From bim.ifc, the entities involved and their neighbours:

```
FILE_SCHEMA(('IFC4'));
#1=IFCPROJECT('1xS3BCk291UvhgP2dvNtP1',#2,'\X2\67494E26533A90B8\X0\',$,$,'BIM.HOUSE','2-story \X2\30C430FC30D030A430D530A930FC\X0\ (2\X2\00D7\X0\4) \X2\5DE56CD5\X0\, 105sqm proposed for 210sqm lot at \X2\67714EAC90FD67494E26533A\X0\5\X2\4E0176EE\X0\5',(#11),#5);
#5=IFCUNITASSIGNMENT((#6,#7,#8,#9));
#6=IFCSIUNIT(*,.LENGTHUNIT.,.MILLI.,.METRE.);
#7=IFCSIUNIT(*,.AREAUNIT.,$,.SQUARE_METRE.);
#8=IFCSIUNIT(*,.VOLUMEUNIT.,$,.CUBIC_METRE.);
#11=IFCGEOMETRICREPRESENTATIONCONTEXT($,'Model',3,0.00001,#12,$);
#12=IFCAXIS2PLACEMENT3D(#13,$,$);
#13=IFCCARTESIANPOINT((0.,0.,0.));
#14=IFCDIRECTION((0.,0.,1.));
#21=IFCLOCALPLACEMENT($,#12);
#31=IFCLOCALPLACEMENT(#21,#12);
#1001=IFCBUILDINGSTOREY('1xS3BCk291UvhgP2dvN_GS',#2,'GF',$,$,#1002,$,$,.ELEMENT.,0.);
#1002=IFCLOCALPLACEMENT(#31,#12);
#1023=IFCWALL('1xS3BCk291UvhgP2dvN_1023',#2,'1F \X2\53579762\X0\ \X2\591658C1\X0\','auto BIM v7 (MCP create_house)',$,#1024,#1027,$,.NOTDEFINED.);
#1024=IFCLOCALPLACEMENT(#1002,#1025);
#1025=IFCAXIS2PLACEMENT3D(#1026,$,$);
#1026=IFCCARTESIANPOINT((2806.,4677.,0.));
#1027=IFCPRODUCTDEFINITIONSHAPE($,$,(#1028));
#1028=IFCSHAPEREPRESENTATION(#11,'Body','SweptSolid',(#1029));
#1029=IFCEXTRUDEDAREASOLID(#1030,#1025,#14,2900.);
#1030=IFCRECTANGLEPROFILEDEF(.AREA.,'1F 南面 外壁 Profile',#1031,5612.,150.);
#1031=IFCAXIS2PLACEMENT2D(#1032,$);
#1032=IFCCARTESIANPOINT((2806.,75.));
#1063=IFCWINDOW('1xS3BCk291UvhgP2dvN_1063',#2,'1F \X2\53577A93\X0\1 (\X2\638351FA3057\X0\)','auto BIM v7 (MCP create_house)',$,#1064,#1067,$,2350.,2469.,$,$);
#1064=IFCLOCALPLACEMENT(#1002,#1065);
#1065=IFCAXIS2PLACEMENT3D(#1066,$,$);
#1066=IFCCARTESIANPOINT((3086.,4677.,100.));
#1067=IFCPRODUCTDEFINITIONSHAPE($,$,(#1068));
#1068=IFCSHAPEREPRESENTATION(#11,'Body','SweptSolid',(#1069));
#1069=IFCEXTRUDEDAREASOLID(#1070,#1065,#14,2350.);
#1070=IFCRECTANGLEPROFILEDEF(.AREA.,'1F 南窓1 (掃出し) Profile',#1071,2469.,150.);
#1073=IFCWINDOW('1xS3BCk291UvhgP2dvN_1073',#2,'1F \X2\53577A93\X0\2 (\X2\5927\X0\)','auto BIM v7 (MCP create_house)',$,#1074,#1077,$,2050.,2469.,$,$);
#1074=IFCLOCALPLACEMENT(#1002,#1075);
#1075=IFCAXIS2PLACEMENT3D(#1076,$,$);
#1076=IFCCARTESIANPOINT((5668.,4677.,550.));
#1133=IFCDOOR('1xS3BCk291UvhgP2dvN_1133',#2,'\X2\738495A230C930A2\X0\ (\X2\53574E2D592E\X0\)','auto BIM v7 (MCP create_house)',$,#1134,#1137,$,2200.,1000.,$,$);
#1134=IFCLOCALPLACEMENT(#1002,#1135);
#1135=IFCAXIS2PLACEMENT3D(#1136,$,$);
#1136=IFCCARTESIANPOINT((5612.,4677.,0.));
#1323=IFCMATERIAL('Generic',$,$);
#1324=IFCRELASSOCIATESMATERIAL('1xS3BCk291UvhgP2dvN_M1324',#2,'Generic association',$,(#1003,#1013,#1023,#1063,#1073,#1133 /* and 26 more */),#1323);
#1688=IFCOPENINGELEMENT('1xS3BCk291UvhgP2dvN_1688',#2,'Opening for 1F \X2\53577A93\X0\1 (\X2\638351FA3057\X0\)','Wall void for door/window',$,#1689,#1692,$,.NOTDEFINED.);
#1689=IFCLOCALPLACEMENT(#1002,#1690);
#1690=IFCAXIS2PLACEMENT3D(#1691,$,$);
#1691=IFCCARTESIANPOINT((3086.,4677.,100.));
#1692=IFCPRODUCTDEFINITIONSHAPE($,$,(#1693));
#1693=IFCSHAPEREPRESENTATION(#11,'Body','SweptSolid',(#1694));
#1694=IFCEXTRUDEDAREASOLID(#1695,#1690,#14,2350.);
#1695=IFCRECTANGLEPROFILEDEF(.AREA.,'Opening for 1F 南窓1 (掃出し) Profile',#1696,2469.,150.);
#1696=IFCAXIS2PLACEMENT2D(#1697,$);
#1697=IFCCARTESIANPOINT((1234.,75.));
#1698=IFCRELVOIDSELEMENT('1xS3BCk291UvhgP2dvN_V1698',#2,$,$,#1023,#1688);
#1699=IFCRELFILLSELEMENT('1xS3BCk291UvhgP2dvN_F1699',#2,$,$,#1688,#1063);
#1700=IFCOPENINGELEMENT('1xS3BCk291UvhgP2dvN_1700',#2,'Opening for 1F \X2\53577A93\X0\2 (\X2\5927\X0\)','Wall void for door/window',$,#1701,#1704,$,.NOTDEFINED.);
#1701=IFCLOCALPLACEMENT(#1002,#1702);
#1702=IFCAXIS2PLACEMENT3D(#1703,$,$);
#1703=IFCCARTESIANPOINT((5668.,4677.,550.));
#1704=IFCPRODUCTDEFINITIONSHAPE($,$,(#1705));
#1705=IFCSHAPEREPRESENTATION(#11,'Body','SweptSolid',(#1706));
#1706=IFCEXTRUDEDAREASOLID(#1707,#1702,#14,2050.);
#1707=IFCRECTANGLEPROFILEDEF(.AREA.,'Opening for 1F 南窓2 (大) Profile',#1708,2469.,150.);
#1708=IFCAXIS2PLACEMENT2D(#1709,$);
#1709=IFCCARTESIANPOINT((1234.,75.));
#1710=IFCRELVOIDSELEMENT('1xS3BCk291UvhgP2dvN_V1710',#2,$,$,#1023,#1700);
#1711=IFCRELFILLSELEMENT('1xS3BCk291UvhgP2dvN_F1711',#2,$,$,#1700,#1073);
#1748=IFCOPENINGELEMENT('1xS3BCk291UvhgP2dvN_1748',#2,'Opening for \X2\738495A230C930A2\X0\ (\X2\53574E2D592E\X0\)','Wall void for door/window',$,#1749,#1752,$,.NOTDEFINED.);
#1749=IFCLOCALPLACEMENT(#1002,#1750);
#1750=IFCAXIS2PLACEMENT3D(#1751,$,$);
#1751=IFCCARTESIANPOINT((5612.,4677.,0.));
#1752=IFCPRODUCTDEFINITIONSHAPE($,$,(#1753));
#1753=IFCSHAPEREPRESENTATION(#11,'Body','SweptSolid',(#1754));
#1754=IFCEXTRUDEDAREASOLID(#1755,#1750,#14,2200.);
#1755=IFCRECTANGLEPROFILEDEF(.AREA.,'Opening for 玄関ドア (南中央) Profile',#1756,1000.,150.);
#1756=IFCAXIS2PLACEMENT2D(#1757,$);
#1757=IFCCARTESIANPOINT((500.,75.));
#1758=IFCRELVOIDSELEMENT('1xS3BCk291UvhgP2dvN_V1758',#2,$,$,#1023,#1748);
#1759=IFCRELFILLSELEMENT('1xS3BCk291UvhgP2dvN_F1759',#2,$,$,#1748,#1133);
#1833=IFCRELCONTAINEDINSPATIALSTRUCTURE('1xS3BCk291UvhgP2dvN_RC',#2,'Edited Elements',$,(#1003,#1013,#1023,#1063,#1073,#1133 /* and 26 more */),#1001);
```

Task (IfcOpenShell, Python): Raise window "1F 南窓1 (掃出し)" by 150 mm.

```python
import numpy as np
import ifcopenshell
import ifcopenshell.api.geometry
import ifcopenshell.util.placement
import ifcopenshell.util.unit

model = ifcopenshell.open("bim.ifc")
unit_scale = ifcopenshell.util.unit.calculate_unit_scale(model)

window = model.by_guid("1xS3BCk291UvhgP2dvN_1063")
opening = window.FillsVoids[0].RelatingOpeningElement
dz = 150.0

shift = np.array([0.0, 0.0, dz])
# The window is not placed relative to its opening, so move both.
for product in (opening, window):
    matrix = ifcopenshell.util.placement.get_local_placement(product.ObjectPlacement)
    matrix[:3, 3] += shift
    ifcopenshell.api.geometry.edit_object_placement(model, product=product, matrix=matrix, is_si=False)

print(f"moved by {dz * unit_scale:+.3f} m")

model.write("bim_rev.ifc")
```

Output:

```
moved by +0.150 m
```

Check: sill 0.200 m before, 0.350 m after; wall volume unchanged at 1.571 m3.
